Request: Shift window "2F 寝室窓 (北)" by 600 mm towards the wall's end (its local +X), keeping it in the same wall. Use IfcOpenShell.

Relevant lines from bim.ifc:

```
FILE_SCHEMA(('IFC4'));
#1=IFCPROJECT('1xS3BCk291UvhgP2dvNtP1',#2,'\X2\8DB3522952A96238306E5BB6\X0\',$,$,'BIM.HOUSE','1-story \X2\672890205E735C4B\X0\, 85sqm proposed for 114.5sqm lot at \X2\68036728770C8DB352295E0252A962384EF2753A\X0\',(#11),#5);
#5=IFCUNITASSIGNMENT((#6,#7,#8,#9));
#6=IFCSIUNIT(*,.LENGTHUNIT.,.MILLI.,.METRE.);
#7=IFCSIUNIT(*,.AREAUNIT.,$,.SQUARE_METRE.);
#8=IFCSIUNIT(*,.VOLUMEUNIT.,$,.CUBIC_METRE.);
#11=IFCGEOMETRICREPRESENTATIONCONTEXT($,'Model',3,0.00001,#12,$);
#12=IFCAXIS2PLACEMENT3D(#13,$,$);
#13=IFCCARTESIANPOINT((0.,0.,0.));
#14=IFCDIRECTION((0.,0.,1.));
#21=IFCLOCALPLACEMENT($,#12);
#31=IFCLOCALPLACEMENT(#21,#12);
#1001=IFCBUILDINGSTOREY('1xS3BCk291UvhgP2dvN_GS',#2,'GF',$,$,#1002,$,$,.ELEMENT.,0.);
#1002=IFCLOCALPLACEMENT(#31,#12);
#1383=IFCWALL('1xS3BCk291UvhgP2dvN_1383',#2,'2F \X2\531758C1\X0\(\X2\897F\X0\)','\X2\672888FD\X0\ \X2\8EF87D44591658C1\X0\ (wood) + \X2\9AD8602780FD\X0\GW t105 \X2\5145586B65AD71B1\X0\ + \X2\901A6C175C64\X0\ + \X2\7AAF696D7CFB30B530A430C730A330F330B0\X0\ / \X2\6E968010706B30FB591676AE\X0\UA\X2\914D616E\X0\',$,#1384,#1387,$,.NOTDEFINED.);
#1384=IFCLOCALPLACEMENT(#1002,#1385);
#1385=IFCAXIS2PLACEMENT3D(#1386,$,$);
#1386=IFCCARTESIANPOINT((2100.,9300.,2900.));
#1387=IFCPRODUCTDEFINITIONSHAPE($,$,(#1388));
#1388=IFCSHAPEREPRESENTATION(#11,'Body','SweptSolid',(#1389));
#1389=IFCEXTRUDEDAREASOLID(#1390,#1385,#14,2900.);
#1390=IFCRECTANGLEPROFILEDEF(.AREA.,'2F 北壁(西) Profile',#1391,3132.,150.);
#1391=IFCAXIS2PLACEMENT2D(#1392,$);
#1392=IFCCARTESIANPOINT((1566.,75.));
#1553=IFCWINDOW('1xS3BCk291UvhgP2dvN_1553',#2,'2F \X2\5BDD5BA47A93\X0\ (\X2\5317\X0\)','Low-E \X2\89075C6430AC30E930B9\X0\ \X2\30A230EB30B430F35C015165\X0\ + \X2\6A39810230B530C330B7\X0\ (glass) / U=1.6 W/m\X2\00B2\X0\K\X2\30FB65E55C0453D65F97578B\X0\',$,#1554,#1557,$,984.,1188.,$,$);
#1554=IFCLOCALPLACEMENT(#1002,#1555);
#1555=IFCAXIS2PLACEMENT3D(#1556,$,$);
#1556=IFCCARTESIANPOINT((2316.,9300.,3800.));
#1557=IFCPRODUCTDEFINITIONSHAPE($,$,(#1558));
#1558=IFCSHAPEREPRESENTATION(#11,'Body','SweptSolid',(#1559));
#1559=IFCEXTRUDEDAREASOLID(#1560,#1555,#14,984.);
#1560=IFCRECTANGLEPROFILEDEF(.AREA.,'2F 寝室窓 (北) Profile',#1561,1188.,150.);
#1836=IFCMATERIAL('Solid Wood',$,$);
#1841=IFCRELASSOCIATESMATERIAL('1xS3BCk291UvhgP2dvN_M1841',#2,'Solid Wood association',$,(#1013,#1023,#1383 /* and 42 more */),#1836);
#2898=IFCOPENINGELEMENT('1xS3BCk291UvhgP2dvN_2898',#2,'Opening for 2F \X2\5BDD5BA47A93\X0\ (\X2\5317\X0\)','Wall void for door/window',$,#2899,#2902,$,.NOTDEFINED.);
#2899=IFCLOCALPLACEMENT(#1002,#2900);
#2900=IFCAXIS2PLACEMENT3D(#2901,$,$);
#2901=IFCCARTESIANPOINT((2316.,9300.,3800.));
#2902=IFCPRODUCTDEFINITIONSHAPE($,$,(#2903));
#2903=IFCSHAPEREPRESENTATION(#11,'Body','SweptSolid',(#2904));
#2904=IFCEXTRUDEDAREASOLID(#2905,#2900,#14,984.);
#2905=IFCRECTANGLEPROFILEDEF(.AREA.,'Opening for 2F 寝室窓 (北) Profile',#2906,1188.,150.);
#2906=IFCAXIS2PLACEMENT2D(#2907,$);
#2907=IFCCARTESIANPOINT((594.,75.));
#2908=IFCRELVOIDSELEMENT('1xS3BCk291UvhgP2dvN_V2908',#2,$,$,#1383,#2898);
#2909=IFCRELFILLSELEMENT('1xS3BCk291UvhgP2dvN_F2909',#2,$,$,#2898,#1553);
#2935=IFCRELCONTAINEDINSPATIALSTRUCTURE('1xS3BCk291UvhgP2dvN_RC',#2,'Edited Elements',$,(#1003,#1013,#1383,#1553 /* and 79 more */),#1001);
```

```python
import ifcopenshell
import ifcopenshell.api.geometry
import ifcopenshell.util.placement

model = ifcopenshell.open("bim.ifc")

window = model.by_guid("1xS3BCk291UvhgP2dvN_1553")
opening = window.FillsVoids[0].RelatingOpeningElement
wall = opening.VoidsElements[0].RelatingBuildingElement

wall_matrix = ifcopenshell.util.placement.get_local_placement(wall.ObjectPlacement)
shift = wall_matrix[:3, 0] * 600.0
before = ifcopenshell.util.placement.get_local_placement(window.ObjectPlacement)[:3, 3].copy()

# The window is not placed relative to its opening, so move both.
for product in (opening, window):
    matrix = ifcopenshell.util.placement.get_local_placement(product.ObjectPlacement)
    matrix[:3, 3] += shift
    ifcopenshell.api.geometry.edit_object_placement(model, product=product, matrix=matrix, is_si=False)

after = ifcopenshell.util.placement.get_local_placement(window.ObjectPlacement)[:3, 3]
print("window moved by", (after - before).round(3) + 0.0)

model.write("bim_rev.ifc")
```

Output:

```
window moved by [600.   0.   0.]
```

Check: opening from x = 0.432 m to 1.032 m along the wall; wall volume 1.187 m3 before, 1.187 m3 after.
